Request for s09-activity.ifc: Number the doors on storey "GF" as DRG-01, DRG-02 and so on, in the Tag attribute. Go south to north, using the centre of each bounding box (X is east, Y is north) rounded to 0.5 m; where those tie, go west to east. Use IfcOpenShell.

First a look at what the model holds.

```python
import ifcopenshell
import ifcopenshell.util.element
import ifcopenshell.util.placement

model = ifcopenshell.open("s09-activity.ifc")
print(model.schema)
storey = next(s for s in model.by_type("IfcBuildingStorey") if s.Name == "GF")
doors = [e for e in ifcopenshell.util.element.get_decomposition(storey) if e.is_a("IfcDoor")]
for e in sorted(doors, key=lambda e: e.id()):
    origin = ifcopenshell.util.placement.get_local_placement(e.ObjectPlacement)[:3, 3]
    print(e.id(), e.Tag, e.Name, origin.round(2) + 0.0, sep=" | ")
```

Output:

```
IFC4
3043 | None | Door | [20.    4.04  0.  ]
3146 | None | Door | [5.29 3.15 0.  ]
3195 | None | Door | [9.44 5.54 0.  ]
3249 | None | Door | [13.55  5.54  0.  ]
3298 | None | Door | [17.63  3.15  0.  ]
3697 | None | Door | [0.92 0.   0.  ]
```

```python
import ifcopenshell
import ifcopenshell.geom
import ifcopenshell.util.element
import ifcopenshell.util.shape

model = ifcopenshell.open("s09-activity.ifc")
settings = ifcopenshell.geom.settings()
settings.set("use-world-coords", True)


def centre(element):
    shape = ifcopenshell.geom.create_shape(settings, element)
    return ifcopenshell.util.shape.get_bbox_centroid(shape.geometry)


storey = next(s for s in model.by_type("IfcBuildingStorey") if s.Name == "GF")
doors = [e for e in ifcopenshell.util.element.get_decomposition(storey) if e.is_a("IfcDoor")]

# Insertion points can sit at a corner or the storey origin, so sort by the geometry (in metres).
centres = {e: centre(e) for e in doors}
doors.sort(key=lambda e: (round(centres[e][1] / 0.5), centres[e][0]))

for i, e in enumerate(doors, start=1):
    number = f"DRG-{i:02d}"
    e.Tag = number
    print(e.id(), number)

model.write("s09-activity_updated.ifc")
```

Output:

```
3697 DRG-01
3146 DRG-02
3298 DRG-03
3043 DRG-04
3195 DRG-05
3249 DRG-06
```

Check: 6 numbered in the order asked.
